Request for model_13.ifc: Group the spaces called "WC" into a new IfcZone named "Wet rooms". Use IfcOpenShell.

First a look at what the model holds.

```python
import ifcopenshell

model = ifcopenshell.open("model_13.ifc")
print(model.schema)
seen = {}
for space in model.by_type("IfcSpace"):
    seen[space.LongName] = seen.get(space.LongName, 0) + 1
for name, count in sorted(seen.items(), key=str):
    print(count, "x", name)
print("zones:", [z.Name for z in model.by_type("IfcZone")][:20])
```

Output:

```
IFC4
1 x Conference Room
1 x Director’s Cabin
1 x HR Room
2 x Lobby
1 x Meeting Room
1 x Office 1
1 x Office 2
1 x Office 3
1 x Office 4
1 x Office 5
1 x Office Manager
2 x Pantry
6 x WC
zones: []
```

```python
import ifcopenshell
import ifcopenshell.api.group
import ifcopenshell.api.root

model = ifcopenshell.open("model_13.ifc")

names = {"WC"}
spaces = [s for s in model.by_type("IfcSpace") if s.LongName in names]

zone = ifcopenshell.api.root.create_entity(model, ifc_class="IfcZone", name="Wet rooms")
ifcopenshell.api.group.assign_group(model, products=spaces, group=zone)
print(len(spaces), "spaces in", zone.Name)

model.write("model_13_rev.ifc")
```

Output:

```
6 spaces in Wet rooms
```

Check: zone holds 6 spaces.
